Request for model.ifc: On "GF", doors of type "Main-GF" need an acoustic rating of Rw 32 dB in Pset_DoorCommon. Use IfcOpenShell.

First a look at what the model holds.

```python
import ifcopenshell
import ifcopenshell.util.element

model = ifcopenshell.open("model.ifc")
print(model.schema)
storey = next(s for s in model.by_type("IfcBuildingStorey") if s.Name == "GF")
doors = [e for e in ifcopenshell.util.element.get_decomposition(storey) if e.is_a("IfcDoor")]
seen = {}
for e in doors:
    element_type = ifcopenshell.util.element.get_type(e)
    key = (element_type.Name if element_type != e and element_type else None, ifcopenshell.util.element.get_pset(e, "Pset_DoorCommon", "AcousticRating"))
    seen[key] = seen.get(key, 0) + 1
for (name, value), count in sorted(seen.items(), key=str):
    print(count, "x", name, "|", value)
```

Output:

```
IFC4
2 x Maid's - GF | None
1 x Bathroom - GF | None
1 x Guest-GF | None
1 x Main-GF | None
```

```python
import ifcopenshell
import ifcopenshell.api.pset
import ifcopenshell.util.element

model = ifcopenshell.open("model.ifc")

storey = next(s for s in model.by_type("IfcBuildingStorey") if s.Name == "GF")
doors = [e for e in ifcopenshell.util.element.get_decomposition(storey) if e.is_a("IfcDoor")]

count = 0
for e in doors:
    element_type = ifcopenshell.util.element.get_type(e)
    if element_type in (None, e) or element_type.Name != "Main-GF":
        continue
    # add_pset returns the element's existing set when there is one.
    pset = ifcopenshell.api.pset.add_pset(model, product=e, name="Pset_DoorCommon")
    ifcopenshell.api.pset.edit_pset(model, pset=pset, properties={"AcousticRating": "Rw 32 dB"})
    count += 1

print(count, "doors updated")

model.write("model_edited.ifc")
```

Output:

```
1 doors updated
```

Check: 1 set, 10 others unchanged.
